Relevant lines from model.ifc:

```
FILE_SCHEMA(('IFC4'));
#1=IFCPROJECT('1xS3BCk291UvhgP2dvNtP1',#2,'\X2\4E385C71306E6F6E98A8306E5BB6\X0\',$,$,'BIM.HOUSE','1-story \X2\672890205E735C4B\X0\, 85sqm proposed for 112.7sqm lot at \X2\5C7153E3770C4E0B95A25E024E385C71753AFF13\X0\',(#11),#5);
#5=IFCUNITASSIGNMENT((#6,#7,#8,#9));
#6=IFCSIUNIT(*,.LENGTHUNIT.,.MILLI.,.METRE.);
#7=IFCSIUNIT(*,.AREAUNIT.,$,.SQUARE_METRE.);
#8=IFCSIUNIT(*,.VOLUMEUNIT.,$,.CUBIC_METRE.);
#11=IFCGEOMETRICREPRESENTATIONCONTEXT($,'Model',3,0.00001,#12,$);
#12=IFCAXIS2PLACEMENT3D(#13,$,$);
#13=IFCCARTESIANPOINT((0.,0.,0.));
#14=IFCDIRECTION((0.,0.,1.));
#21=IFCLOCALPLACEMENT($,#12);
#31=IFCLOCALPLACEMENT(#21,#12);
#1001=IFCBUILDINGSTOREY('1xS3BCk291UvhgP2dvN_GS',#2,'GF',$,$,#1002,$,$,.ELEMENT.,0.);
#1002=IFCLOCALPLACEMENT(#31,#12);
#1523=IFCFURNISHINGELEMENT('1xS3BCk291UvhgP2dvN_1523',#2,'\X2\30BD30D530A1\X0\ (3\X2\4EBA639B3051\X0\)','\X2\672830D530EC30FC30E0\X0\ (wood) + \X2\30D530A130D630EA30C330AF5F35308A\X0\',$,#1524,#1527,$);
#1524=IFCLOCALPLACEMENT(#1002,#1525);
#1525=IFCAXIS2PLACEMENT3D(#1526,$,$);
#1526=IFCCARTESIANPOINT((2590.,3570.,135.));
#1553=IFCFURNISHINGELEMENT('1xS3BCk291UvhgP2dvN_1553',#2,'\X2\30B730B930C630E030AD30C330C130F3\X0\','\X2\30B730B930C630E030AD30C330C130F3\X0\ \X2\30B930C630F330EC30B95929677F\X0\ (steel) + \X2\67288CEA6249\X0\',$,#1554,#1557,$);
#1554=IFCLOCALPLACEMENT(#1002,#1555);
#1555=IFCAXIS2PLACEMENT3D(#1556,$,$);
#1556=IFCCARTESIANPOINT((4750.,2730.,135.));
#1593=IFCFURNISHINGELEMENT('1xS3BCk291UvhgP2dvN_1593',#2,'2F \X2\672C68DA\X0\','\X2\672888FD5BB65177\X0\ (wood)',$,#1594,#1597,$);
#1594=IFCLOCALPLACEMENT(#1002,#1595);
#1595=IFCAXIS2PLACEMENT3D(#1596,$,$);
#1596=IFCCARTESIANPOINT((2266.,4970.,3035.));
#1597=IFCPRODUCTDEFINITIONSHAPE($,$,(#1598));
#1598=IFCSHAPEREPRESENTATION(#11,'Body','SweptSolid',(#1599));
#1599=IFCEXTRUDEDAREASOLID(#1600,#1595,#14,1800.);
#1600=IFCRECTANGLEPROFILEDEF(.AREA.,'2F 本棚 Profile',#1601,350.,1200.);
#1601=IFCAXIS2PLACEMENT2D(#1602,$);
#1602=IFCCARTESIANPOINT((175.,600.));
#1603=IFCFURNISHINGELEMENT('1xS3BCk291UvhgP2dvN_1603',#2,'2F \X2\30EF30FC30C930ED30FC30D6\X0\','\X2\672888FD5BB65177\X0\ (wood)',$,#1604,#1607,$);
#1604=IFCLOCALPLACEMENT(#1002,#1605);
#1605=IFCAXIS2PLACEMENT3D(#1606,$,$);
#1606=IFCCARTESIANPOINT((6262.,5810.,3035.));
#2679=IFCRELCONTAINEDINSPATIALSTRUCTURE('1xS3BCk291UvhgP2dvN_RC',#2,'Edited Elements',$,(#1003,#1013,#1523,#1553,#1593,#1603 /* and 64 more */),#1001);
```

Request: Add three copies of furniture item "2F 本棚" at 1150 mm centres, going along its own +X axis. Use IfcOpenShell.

```python
import ifcopenshell
import ifcopenshell.api.geometry
import ifcopenshell.api.root
import ifcopenshell.util.element
import ifcopenshell.util.placement

model = ifcopenshell.open("model.ifc")


def reuse_history(source, copy):
    """copy_class also copies each property set's owner history, people and application; keep the originals."""
    for rel in copy.IsDefinedBy:
        if rel.is_a("IfcRelDefinesByProperties") and (history := rel.RelatingPropertyDefinition.OwnerHistory):
            rel.RelatingPropertyDefinition.OwnerHistory = source.OwnerHistory
            ifcopenshell.util.element.remove_deep2(model, history)


source = model.by_guid("1xS3BCk291UvhgP2dvN_1593")
base = ifcopenshell.util.placement.get_local_placement(source.ObjectPlacement)
step = base[:3, 0] * 1150.0

for i in range(1, 4):
    copy = ifcopenshell.api.root.copy_class(model, product=source)
    copy.Representation = ifcopenshell.util.element.copy_deep(
        model, source.Representation, exclude=["IfcGeometricRepresentationContext", "IfcRepresentationMap"]
    )
    reuse_history(source, copy)
    matrix = base.copy()
    matrix[:3, 3] += i * step
    print("added at", matrix[:3, 3].round(3) + 0.0)
    ifcopenshell.api.geometry.edit_object_placement(model, product=copy, matrix=matrix, is_si=False)

model.write("model-out.ifc")
```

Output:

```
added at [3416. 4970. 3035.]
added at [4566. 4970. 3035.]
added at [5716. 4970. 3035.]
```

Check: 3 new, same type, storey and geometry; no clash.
